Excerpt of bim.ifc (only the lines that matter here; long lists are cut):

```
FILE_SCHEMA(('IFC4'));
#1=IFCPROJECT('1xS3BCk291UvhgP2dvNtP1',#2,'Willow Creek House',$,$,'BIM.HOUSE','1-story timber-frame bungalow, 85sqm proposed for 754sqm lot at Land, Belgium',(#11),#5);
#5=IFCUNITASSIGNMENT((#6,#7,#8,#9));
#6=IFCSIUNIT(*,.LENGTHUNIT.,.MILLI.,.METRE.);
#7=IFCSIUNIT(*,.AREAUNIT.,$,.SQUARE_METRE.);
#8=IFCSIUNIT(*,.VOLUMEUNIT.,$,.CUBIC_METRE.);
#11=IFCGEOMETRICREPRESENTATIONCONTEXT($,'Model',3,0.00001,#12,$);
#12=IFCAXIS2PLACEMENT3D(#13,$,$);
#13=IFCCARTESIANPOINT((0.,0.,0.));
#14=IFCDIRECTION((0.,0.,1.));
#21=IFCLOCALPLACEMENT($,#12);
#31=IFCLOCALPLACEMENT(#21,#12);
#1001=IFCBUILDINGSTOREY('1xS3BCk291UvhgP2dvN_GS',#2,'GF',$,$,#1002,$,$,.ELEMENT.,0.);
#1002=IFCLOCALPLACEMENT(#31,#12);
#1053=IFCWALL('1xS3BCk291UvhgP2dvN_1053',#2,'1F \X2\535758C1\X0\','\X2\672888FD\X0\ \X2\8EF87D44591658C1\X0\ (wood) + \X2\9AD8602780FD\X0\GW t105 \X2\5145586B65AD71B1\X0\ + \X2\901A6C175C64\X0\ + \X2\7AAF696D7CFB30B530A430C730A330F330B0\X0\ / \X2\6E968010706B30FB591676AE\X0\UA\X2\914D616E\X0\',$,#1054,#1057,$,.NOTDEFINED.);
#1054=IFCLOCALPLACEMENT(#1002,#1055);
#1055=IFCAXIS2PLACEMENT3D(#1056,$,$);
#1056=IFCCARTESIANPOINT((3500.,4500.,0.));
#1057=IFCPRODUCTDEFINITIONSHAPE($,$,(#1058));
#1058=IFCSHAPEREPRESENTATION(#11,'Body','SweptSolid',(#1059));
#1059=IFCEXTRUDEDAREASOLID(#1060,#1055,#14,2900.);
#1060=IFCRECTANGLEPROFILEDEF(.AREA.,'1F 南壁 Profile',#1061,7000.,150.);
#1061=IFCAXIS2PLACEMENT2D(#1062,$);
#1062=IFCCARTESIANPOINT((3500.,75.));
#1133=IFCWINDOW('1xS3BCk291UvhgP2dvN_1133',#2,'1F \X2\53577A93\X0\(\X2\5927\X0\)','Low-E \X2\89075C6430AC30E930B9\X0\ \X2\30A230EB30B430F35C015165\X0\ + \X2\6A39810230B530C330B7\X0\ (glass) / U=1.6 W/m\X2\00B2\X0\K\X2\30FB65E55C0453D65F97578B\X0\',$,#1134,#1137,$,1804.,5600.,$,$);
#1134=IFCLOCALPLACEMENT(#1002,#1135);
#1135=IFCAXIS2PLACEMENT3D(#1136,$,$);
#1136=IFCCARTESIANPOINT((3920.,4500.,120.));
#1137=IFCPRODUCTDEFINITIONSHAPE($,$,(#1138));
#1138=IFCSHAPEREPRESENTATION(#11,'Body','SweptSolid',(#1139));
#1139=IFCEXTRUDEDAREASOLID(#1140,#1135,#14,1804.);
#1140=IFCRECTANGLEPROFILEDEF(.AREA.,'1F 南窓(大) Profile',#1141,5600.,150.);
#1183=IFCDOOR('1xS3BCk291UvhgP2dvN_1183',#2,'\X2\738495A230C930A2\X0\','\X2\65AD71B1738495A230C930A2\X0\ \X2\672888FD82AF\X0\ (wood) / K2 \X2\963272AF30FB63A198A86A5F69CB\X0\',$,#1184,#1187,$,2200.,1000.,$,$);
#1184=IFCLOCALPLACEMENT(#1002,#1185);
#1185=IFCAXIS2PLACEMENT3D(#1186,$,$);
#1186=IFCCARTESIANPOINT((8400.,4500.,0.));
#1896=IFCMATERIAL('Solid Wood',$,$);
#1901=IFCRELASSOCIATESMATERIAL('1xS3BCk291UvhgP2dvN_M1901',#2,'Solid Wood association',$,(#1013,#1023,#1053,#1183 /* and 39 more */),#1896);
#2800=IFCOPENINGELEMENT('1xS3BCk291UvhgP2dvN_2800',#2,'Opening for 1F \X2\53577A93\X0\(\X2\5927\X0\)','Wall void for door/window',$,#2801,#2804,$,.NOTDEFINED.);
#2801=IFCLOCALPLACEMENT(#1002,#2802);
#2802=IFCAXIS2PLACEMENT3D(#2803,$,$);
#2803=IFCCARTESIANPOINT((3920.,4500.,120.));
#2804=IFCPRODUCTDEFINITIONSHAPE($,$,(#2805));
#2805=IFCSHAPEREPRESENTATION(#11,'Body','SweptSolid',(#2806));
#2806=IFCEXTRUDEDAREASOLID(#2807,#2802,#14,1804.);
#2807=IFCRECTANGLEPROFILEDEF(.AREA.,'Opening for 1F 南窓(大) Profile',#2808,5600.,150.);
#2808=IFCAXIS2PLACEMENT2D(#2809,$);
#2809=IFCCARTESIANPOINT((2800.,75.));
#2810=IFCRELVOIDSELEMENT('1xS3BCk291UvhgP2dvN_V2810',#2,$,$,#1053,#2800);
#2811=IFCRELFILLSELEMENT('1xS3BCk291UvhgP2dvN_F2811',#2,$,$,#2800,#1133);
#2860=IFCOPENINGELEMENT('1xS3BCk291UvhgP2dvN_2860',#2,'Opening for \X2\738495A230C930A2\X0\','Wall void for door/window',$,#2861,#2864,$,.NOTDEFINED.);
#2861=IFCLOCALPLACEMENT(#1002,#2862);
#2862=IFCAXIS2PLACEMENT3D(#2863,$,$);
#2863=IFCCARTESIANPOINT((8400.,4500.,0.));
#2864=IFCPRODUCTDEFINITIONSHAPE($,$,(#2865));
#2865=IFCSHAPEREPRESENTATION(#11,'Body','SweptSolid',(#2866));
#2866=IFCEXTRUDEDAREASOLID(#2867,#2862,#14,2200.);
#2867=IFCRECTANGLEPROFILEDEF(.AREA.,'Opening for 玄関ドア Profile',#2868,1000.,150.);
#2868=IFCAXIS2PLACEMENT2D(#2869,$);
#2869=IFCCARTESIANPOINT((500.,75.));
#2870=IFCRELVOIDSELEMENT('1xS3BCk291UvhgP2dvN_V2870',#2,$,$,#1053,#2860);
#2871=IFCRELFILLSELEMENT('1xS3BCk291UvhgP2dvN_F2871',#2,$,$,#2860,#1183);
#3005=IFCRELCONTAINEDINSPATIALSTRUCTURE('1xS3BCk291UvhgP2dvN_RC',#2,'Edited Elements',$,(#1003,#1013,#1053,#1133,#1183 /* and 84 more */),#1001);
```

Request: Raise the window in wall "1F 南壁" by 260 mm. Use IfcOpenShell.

```python
import numpy as np
import ifcopenshell
import ifcopenshell.api.geometry
import ifcopenshell.util.placement
import ifcopenshell.util.unit

model = ifcopenshell.open("bim.ifc")
unit_scale = ifcopenshell.util.unit.calculate_unit_scale(model)

window = model.by_guid("1xS3BCk291UvhgP2dvN_1133")
opening = window.FillsVoids[0].RelatingOpeningElement
dz = 0.26 / unit_scale

shift = np.array([0.0, 0.0, dz])
# The window is not placed relative to its opening, so move both.
for product in (opening, window):
    matrix = ifcopenshell.util.placement.get_local_placement(product.ObjectPlacement)
    matrix[:3, 3] += shift
    ifcopenshell.api.geometry.edit_object_placement(model, product=product, matrix=matrix, is_si=False)

print(f"moved by {dz * unit_scale:+.3f} m")

model.write("bim_edited.ifc")
```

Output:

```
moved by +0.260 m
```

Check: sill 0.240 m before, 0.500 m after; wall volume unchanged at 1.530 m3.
